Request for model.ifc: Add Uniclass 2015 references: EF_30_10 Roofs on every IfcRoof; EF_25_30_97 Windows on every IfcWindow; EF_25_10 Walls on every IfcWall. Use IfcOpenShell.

First a look at what the model holds.

```python
import ifcopenshell

model = ifcopenshell.open("model.ifc")
print(model.schema)
print("classifications:", [c.Name for c in model.by_type("IfcClassification")])
for ifc_class in ("IfcDoor", "IfcRoof", "IfcStair", "IfcWall", "IfcWindow"):
    print(ifc_class, len(model.by_type(ifc_class)))
```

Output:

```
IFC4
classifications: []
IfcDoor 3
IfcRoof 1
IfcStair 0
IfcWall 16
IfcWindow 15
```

```python
import ifcopenshell
import ifcopenshell.api.classification

model = ifcopenshell.open("model.ifc")

system = ifcopenshell.api.classification.add_classification(model, classification="Uniclass 2015")

codes = {
    "IfcRoof": ("EF_30_10", "Roofs"),
    "IfcWindow": ("EF_25_30_97", "Windows"),
    "IfcWall": ("EF_25_10", "Walls"),
}
for ifc_class, (code, name) in codes.items():
    products = model.by_type(ifc_class)
    ifcopenshell.api.classification.add_reference(
        model, products=products, classification=system, identification=code, name=name
    )
    print(code, len(products))

model.write("model_rev.ifc")
```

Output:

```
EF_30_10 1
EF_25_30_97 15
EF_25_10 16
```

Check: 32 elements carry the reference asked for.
